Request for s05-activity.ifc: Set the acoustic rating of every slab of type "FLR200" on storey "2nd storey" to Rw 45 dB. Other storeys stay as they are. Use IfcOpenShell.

First a look at what the model holds.

```python
import ifcopenshell
import ifcopenshell.util.element

model = ifcopenshell.open("s05-activity.ifc")
print(model.schema)
storey = next(s for s in model.by_type("IfcBuildingStorey") if s.Name == "2nd storey")
slabs = [e for e in ifcopenshell.util.element.get_decomposition(storey) if e.is_a("IfcSlab")]
seen = {}
for e in slabs:
    element_type = ifcopenshell.util.element.get_type(e)
    key = (element_type.Name if element_type != e and element_type else None, ifcopenshell.util.element.get_pset(e, "Pset_SlabCommon", "AcousticRating"))
    seen[key] = seen.get(key, 0) + 1
for (name, value), count in sorted(seen.items(), key=str):
    print(count, "x", name, "|", value)
```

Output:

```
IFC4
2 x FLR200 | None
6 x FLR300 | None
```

```python
import ifcopenshell
import ifcopenshell.api.pset
import ifcopenshell.util.element

model = ifcopenshell.open("s05-activity.ifc")

storey = next(s for s in model.by_type("IfcBuildingStorey") if s.Name == "2nd storey")
slabs = [e for e in ifcopenshell.util.element.get_decomposition(storey) if e.is_a("IfcSlab")]

count = 0
for e in slabs:
    element_type = ifcopenshell.util.element.get_type(e)
    if element_type in (None, e) or element_type.Name != "FLR200":
        continue
    # add_pset returns the element's existing set when there is one.
    pset = ifcopenshell.api.pset.add_pset(model, product=e, name="Pset_SlabCommon")
    ifcopenshell.api.pset.edit_pset(model, pset=pset, properties={"AcousticRating": "Rw 45 dB"})
    count += 1

print(count, "slabs updated")

model.write("s05-activity-out.ifc")
```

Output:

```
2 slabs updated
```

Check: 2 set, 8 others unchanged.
